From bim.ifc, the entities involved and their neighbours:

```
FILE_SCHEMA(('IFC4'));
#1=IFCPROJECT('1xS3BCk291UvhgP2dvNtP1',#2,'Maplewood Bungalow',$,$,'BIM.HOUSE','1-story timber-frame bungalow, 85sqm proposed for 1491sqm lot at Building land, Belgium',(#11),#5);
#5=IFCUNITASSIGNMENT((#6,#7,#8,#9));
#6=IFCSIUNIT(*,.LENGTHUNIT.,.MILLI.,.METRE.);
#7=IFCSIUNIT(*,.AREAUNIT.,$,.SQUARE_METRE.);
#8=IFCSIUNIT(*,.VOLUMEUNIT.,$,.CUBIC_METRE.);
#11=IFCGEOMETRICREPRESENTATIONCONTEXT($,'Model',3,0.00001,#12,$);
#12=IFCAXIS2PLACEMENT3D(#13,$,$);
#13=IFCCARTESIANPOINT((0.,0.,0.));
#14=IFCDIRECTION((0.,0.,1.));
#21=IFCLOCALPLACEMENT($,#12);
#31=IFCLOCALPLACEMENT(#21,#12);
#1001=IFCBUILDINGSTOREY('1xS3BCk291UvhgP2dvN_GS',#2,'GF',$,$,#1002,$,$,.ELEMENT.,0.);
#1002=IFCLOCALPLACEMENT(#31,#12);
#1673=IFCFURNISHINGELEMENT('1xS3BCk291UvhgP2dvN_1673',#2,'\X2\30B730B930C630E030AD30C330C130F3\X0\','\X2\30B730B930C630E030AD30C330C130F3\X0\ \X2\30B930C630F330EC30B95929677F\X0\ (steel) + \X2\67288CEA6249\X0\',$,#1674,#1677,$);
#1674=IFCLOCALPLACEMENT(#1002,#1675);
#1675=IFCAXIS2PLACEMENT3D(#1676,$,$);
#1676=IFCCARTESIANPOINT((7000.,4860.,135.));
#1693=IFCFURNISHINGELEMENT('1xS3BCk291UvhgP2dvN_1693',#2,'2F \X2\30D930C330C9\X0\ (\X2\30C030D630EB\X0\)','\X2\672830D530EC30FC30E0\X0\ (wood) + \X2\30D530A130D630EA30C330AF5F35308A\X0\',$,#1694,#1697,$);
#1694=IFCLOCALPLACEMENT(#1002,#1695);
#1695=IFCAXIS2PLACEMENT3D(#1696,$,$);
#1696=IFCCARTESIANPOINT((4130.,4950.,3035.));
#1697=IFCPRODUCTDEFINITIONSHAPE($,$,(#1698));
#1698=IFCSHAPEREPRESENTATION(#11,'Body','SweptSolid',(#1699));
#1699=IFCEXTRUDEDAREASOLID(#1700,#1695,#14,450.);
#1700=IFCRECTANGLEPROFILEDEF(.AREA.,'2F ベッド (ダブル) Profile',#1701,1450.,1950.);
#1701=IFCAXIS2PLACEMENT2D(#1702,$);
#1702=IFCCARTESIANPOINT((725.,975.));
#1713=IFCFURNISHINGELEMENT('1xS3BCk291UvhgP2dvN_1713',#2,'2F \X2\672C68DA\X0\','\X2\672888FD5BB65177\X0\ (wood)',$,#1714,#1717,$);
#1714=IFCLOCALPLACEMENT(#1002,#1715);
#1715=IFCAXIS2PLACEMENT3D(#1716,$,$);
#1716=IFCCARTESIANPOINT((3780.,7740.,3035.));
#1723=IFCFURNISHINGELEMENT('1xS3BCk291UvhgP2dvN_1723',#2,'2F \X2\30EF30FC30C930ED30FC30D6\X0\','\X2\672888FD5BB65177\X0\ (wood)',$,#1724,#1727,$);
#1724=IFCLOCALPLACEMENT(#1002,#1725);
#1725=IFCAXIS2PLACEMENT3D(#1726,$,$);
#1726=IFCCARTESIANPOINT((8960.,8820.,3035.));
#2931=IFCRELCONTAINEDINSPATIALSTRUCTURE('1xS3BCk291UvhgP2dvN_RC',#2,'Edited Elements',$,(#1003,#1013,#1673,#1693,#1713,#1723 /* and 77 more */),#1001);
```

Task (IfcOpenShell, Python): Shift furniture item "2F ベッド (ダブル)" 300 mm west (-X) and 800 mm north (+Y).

```python
import ifcopenshell
import ifcopenshell.api.geometry
import ifcopenshell.util.placement

model = ifcopenshell.open("bim.ifc")

item = model.by_id(1693)
matrix = ifcopenshell.util.placement.get_local_placement(item.ObjectPlacement)
matrix[0, 3] -= 300.0
matrix[1, 3] += 800.0
ifcopenshell.api.geometry.edit_object_placement(model, product=item, matrix=matrix, is_si=False)

print(ifcopenshell.util.placement.get_local_placement(item.ObjectPlacement).round(3) + 0.0)

model.write("bim_v2.ifc")
```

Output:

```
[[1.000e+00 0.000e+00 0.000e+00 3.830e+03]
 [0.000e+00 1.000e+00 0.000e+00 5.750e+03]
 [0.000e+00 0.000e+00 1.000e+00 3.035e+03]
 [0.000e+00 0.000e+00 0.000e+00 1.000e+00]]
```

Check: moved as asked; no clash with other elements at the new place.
